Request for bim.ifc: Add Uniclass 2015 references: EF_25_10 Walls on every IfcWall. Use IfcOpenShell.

First a look at what the model holds.

```python
import ifcopenshell

model = ifcopenshell.open("bim.ifc")
print(model.schema)
print("classifications:", [c.Name for c in model.by_type("IfcClassification")])
for ifc_class in ("IfcDoor", "IfcRoof", "IfcStair", "IfcWall", "IfcWindow"):
    print(ifc_class, len(model.by_type(ifc_class)))
```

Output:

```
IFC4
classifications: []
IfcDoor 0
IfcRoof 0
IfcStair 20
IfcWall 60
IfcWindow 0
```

```python
import ifcopenshell
import ifcopenshell.api.classification

model = ifcopenshell.open("bim.ifc")

system = ifcopenshell.api.classification.add_classification(model, classification="Uniclass 2015")

codes = {
    "IfcWall": ("EF_25_10", "Walls"),
}
for ifc_class, (code, name) in codes.items():
    products = model.by_type(ifc_class)
    ifcopenshell.api.classification.add_reference(
        model, products=products, classification=system, identification=code, name=name
    )
    print(code, len(products))

model.write("bim-out.ifc")
```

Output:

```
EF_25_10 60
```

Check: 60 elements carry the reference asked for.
